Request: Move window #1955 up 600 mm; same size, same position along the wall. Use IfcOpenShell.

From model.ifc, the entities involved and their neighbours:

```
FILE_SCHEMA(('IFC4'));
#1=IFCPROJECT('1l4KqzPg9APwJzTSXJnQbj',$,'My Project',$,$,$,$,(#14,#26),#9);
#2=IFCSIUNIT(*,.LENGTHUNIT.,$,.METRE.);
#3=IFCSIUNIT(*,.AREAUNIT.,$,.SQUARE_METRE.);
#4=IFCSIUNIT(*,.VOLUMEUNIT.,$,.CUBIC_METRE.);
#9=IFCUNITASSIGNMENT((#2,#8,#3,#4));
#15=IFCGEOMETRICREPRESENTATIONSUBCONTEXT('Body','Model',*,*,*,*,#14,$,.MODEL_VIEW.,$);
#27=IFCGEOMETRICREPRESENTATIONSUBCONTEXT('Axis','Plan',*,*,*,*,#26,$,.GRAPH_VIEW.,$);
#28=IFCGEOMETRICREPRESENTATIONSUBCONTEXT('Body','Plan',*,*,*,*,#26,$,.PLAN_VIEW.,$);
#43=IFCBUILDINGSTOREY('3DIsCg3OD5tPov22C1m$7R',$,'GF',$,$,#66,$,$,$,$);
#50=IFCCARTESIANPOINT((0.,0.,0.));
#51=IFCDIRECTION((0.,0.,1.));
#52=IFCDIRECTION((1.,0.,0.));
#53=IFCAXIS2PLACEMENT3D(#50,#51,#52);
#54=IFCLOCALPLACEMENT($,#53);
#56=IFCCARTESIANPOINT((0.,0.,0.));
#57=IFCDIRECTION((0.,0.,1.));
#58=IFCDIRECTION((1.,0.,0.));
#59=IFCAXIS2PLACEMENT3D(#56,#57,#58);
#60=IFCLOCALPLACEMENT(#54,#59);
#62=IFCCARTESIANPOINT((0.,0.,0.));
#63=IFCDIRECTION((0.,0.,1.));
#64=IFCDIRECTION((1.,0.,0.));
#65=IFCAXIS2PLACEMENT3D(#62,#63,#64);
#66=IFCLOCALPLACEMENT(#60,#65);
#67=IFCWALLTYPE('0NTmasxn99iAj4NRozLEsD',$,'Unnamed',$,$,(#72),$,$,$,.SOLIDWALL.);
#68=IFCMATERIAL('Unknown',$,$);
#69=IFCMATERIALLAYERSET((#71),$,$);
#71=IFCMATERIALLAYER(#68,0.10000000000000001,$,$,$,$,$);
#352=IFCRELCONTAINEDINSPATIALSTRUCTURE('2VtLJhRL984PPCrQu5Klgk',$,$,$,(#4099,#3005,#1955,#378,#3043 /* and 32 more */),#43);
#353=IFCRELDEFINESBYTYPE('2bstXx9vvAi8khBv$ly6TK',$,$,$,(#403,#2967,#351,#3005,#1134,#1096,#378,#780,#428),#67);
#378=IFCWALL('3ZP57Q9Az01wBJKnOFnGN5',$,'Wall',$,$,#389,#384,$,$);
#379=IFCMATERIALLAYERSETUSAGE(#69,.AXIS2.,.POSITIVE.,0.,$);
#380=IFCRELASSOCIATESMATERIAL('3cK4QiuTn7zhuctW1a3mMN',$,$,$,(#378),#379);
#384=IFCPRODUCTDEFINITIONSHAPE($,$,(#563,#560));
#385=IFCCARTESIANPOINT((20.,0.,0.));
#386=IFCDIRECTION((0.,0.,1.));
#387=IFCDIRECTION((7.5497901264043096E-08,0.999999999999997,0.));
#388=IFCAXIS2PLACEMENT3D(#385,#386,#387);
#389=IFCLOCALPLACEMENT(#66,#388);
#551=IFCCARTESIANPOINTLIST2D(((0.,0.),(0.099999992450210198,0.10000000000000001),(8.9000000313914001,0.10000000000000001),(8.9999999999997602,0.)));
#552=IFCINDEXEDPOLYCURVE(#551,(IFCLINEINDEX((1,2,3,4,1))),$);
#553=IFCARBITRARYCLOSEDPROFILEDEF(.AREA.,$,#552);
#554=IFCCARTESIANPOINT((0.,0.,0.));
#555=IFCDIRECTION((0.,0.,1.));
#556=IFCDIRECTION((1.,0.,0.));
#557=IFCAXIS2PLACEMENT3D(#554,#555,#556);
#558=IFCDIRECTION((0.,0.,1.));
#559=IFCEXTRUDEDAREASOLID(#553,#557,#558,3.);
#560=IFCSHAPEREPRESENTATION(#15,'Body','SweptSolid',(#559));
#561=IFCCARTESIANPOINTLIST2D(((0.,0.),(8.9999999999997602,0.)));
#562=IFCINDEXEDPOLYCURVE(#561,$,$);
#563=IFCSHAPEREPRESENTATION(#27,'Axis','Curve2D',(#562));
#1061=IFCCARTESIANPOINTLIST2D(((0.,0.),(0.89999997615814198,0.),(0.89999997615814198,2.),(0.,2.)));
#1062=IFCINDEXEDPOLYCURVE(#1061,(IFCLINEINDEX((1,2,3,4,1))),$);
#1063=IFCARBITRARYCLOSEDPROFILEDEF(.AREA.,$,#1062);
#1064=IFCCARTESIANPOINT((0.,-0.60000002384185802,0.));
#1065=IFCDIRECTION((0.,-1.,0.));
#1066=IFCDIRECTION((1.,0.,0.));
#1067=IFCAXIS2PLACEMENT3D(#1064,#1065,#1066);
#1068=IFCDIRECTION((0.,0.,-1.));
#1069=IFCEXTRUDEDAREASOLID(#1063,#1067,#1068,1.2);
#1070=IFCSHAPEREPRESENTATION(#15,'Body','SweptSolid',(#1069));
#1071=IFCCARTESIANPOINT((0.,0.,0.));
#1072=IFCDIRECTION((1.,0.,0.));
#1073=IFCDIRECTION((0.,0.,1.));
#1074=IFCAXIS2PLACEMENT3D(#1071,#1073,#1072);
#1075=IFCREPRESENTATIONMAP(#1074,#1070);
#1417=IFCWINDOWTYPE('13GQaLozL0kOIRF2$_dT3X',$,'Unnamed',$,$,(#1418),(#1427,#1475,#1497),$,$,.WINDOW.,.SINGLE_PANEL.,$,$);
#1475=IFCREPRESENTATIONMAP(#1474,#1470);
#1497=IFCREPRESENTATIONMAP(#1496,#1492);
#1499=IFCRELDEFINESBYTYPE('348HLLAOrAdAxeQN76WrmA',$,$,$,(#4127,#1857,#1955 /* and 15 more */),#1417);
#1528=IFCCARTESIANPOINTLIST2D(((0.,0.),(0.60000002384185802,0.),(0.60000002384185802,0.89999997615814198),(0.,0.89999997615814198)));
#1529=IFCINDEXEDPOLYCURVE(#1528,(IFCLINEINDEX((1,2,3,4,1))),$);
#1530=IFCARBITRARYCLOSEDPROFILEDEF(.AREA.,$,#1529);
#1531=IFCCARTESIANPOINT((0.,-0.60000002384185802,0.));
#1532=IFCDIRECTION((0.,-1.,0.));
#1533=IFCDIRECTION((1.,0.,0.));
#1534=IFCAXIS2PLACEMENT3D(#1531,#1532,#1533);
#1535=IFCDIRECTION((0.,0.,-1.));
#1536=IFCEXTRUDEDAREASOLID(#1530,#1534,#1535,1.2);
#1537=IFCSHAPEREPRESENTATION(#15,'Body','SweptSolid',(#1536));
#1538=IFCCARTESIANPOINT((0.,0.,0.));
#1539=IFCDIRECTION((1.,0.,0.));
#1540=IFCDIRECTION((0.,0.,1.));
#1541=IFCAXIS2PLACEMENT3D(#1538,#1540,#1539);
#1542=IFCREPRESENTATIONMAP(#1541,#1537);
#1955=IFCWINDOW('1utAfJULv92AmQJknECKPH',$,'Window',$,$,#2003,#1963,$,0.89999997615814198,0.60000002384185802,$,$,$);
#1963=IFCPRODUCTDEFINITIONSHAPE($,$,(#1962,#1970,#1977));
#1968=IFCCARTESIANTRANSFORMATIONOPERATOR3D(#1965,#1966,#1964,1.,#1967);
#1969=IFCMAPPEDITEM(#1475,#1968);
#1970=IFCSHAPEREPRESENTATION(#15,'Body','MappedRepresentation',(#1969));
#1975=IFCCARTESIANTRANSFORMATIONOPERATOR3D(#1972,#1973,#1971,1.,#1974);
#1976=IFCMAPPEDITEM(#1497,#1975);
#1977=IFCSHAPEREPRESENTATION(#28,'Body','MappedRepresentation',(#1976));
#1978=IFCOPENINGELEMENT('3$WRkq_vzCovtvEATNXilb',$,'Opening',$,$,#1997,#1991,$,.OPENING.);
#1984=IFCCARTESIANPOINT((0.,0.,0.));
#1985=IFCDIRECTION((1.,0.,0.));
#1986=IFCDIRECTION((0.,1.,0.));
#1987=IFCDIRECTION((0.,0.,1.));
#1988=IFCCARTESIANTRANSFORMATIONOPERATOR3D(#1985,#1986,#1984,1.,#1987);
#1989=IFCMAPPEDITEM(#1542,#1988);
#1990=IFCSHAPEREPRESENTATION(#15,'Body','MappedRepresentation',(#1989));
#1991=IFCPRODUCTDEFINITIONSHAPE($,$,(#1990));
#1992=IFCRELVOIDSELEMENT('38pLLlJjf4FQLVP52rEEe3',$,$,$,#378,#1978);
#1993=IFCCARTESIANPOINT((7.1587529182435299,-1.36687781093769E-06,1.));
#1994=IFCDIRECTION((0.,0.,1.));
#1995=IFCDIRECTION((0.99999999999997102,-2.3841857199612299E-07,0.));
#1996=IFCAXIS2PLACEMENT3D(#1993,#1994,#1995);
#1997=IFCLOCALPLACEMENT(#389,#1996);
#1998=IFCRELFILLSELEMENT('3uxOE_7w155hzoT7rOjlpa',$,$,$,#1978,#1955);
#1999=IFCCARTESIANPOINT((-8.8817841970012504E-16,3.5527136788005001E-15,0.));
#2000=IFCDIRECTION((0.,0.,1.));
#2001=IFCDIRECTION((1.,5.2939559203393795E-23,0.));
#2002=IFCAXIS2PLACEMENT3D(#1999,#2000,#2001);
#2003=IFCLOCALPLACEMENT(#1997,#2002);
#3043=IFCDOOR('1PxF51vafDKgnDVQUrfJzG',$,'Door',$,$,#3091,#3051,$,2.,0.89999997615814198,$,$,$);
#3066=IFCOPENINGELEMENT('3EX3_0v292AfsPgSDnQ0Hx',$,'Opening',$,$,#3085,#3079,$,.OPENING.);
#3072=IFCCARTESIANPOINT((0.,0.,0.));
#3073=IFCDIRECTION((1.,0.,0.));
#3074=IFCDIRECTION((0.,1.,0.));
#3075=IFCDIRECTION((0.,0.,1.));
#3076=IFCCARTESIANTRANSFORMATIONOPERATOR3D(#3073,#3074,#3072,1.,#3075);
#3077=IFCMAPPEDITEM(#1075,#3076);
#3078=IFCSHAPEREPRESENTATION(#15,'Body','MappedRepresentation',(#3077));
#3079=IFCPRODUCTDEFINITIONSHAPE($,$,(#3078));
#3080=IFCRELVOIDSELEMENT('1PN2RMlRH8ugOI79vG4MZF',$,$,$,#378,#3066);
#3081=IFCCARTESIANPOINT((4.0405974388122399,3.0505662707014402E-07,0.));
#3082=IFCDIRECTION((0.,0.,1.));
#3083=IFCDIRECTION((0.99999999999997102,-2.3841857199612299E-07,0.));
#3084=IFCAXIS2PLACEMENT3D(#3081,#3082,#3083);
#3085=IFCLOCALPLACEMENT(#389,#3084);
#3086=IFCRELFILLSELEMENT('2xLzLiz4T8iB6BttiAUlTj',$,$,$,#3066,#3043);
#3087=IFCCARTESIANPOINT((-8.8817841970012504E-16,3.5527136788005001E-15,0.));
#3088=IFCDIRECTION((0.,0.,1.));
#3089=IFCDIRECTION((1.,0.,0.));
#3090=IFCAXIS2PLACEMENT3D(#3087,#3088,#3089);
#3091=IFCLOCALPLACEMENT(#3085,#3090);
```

```python
import numpy as np
import ifcopenshell
import ifcopenshell.api.geometry
import ifcopenshell.util.placement
import ifcopenshell.util.unit

model = ifcopenshell.open("model.ifc")
unit_scale = ifcopenshell.util.unit.calculate_unit_scale(model)

window = model.by_guid("1utAfJULv92AmQJknECKPH")
opening = window.FillsVoids[0].RelatingOpeningElement
dz = 0.6 / unit_scale

shift = np.array([0.0, 0.0, dz])
# The window is placed relative to its opening, so it follows when the opening moves.
matrix = ifcopenshell.util.placement.get_local_placement(opening.ObjectPlacement)
matrix[:3, 3] += shift
ifcopenshell.api.geometry.edit_object_placement(
    model, product=opening, matrix=matrix, is_si=False, should_transform_children=True
)

print(f"moved by {dz * unit_scale:+.3f} m")

model.write("model_v2.ifc")
```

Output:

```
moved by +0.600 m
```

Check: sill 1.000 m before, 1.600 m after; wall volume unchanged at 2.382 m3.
